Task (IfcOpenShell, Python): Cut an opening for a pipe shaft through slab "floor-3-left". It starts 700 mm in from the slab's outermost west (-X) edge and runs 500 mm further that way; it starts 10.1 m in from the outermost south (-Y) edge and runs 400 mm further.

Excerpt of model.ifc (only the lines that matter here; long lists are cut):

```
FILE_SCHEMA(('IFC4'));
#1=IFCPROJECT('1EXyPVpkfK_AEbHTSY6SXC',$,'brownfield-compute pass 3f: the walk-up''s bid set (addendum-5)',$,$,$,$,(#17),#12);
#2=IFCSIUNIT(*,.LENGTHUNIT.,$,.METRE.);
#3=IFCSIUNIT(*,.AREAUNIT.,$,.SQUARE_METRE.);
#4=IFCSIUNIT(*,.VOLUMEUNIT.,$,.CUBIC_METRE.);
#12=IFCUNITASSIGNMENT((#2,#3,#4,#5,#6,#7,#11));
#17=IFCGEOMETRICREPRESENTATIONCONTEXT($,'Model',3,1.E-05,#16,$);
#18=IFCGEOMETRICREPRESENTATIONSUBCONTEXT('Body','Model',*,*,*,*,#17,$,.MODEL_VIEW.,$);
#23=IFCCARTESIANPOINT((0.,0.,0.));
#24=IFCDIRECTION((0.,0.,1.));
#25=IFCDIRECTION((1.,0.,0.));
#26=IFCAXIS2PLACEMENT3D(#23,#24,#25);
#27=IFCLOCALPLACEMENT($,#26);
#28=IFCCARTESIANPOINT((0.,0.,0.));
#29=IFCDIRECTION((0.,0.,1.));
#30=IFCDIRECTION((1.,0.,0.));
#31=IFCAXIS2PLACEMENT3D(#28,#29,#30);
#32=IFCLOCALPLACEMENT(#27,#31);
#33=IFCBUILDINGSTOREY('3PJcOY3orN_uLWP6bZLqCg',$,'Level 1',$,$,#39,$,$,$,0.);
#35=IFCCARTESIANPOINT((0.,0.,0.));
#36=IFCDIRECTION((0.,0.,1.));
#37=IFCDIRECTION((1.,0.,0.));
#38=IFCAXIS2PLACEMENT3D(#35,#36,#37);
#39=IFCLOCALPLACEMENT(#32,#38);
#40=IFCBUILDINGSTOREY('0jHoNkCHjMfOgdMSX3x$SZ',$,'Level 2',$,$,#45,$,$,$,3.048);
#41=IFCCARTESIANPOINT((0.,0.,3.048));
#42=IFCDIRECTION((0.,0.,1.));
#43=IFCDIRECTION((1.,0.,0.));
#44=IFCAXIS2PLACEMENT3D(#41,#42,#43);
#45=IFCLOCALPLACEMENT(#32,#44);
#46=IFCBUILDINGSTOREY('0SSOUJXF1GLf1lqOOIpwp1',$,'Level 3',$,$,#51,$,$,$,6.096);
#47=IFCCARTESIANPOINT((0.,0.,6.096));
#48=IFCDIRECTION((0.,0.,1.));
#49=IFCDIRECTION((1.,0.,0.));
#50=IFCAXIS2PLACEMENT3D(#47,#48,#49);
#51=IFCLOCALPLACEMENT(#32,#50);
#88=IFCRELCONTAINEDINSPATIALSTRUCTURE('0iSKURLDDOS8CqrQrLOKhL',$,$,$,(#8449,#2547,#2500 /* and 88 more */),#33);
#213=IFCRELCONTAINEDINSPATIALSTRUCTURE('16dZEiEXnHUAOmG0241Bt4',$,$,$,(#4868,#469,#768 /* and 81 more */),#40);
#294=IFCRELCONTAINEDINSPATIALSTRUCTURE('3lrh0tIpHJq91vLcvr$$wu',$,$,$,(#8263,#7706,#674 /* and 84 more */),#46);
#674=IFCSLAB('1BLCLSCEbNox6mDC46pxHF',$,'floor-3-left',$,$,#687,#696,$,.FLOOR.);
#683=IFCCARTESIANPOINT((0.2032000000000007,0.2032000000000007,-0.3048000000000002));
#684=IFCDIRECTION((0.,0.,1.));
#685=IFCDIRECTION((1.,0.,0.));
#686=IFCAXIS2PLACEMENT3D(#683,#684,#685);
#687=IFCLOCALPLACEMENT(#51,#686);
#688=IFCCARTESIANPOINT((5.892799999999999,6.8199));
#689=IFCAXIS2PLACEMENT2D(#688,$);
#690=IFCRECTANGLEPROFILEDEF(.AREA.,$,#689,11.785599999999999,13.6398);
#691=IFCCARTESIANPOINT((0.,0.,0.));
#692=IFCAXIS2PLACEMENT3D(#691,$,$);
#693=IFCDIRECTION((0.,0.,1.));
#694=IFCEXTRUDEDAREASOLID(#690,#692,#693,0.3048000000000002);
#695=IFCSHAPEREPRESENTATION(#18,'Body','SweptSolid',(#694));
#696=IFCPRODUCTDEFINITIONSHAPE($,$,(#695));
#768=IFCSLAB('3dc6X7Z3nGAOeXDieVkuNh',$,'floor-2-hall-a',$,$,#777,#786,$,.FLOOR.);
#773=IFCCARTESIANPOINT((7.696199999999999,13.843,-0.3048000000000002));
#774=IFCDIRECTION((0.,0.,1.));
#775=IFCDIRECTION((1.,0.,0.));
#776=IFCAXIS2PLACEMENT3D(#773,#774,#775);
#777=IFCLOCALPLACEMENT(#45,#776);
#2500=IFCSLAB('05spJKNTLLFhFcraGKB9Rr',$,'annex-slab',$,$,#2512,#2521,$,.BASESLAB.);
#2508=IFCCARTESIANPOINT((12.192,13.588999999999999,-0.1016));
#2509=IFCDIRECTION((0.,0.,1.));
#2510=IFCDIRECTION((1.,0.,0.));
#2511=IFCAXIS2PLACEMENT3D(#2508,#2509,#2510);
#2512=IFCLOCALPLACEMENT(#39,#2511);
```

```python
import numpy as np
import ifcopenshell
import ifcopenshell.api.feature
import ifcopenshell.api.geometry
import ifcopenshell.api.root
import ifcopenshell.geom
import ifcopenshell.util.placement
import ifcopenshell.util.representation
import ifcopenshell.util.shape
import ifcopenshell.util.unit

model = ifcopenshell.open("model.ifc")
unit_scale = ifcopenshell.util.unit.calculate_unit_scale(model)
settings = ifcopenshell.geom.settings()


def volume(element):
    """Net volume in cubic metres, openings subtracted."""
    shape = ifcopenshell.geom.create_shape(settings, element)
    return ifcopenshell.util.shape.get_volume(shape.geometry)


slab = model.by_guid("1BLCLSCEbNox6mDC46pxHF")
before = volume(slab)

# Extent in the slab's own axes, in metres. The edges named are its -X and -Y sides.
slab_shape = ifcopenshell.geom.create_shape(settings, slab)
vertices = ifcopenshell.util.shape.get_vertices(slab_shape.geometry)
x_min, y_min, bottom = vertices.min(axis=0)
top = vertices[:, 2].max()

opening = ifcopenshell.api.root.create_entity(model, ifc_class="IfcOpeningElement", name="Pipe shaft opening", predefined_type="OPENING")
context = ifcopenshell.util.representation.get_context(model, "Model", "Body", "MODEL_VIEW")
width, depth = 0.5, 0.4
outline = [(0.0, 0.0), (width, 0.0), (width, depth), (0.0, depth), (0.0, 0.0)]
# Overshoot both faces by 50 mm so the cut is clean.
shape = ifcopenshell.api.geometry.add_slab_representation(
    model, context=context, depth=top - bottom + 0.1, polyline=outline
)
ifcopenshell.api.geometry.assign_representation(model, product=opening, representation=shape)

matrix = ifcopenshell.util.placement.get_local_placement(slab.ObjectPlacement)
matrix[:, 3] = matrix @ np.append(np.array([x_min + 0.7, y_min + 10.1, bottom - 0.05]) / unit_scale, 1.0)
ifcopenshell.api.geometry.edit_object_placement(model, product=opening, matrix=matrix, is_si=False)
ifcopenshell.api.feature.add_feature(model, feature=opening, element=slab)

after = volume(slab)

print(f"slab volume {before:.3f} -> {after:.3f} m3")

model.write("model_rev.ifc")
```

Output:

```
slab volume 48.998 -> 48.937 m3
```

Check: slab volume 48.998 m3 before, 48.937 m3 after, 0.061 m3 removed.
